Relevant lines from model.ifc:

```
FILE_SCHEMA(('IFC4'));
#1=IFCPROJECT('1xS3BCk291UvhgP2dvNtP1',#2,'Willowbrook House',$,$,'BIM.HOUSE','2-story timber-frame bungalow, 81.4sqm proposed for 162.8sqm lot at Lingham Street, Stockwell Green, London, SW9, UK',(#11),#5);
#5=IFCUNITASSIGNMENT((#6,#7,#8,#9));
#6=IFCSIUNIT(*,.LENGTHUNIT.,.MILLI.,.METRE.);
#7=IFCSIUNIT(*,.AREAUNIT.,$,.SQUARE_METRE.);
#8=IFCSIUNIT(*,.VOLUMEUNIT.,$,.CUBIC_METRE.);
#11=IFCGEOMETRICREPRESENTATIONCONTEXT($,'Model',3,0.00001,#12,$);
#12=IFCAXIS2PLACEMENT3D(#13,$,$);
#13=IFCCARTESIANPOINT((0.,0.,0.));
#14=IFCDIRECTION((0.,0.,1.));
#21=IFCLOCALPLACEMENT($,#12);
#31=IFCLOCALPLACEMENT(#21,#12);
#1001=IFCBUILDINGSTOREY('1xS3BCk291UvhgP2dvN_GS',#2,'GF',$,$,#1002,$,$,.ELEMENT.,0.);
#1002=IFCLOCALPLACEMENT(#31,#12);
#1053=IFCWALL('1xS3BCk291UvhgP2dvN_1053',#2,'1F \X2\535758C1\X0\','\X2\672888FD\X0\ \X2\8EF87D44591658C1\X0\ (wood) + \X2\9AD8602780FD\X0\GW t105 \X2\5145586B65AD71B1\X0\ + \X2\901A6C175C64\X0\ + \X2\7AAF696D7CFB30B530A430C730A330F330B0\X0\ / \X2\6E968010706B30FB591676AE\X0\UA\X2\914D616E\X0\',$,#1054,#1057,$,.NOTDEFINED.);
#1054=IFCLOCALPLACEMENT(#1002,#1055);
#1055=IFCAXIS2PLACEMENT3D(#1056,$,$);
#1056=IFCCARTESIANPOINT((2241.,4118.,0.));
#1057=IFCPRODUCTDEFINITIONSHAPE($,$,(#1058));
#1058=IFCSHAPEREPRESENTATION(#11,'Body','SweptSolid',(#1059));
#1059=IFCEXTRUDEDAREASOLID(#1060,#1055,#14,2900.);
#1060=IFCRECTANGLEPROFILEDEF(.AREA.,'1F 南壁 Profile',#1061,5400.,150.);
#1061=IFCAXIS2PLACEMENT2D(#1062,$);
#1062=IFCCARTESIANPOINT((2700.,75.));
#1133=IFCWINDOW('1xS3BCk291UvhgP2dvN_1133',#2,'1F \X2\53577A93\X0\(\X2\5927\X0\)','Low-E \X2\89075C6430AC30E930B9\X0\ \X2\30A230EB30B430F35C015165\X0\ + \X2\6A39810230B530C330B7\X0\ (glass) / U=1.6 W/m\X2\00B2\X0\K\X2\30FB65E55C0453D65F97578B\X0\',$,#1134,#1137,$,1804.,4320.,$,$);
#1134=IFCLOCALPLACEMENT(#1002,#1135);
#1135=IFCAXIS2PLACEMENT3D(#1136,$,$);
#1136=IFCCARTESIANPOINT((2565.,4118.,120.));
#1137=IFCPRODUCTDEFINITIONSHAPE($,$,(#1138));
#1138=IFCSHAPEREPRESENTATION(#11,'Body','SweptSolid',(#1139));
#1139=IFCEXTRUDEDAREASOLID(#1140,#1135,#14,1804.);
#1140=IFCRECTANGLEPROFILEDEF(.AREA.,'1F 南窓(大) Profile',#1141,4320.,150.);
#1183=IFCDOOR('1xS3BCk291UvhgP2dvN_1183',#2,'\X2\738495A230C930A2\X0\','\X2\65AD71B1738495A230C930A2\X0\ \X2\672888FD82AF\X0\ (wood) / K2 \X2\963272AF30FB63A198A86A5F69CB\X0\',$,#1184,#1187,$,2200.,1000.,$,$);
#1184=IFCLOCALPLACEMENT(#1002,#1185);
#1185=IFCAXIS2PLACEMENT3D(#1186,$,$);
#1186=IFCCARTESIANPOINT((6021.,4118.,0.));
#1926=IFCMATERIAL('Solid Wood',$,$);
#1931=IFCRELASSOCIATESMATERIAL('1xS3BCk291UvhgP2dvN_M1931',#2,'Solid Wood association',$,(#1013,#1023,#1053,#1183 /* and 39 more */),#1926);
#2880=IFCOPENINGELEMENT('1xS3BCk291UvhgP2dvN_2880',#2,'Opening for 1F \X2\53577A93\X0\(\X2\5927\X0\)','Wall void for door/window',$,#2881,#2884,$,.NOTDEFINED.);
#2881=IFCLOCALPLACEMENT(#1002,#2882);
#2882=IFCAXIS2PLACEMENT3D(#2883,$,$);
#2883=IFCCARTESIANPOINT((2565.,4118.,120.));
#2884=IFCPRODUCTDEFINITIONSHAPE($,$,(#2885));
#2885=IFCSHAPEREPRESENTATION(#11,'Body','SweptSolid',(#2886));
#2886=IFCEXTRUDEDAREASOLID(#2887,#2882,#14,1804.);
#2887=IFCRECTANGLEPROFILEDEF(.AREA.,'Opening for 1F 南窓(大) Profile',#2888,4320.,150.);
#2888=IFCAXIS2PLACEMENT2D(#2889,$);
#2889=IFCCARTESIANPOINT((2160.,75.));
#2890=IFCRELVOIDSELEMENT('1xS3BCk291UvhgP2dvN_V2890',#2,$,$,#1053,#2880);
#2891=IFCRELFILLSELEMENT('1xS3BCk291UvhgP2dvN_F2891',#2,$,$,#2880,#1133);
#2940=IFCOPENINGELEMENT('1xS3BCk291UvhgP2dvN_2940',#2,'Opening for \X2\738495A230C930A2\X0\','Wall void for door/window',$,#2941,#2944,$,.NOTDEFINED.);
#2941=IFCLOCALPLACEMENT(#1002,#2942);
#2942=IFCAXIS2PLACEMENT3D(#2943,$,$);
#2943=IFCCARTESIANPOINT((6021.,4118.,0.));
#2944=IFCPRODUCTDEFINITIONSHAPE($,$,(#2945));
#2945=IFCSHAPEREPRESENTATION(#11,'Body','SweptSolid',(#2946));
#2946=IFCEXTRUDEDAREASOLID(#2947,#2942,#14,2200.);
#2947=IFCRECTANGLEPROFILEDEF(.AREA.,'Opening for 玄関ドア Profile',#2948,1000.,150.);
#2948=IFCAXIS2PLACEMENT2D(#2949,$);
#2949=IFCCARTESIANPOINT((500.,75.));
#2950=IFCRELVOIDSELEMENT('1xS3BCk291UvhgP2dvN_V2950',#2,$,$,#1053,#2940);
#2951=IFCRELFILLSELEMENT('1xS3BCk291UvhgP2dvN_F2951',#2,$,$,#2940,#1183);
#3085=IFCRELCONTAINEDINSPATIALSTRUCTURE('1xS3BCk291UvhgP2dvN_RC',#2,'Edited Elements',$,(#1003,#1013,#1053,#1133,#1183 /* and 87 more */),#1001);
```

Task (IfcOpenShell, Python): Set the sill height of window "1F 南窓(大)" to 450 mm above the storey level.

```python
import numpy as np
import ifcopenshell
import ifcopenshell.api.geometry
import ifcopenshell.geom
import ifcopenshell.util.element
import ifcopenshell.util.placement
import ifcopenshell.util.shape
import ifcopenshell.util.unit

model = ifcopenshell.open("model.ifc")
unit_scale = ifcopenshell.util.unit.calculate_unit_scale(model)

window = model.by_guid("1xS3BCk291UvhgP2dvN_1133")
opening = window.FillsVoids[0].RelatingOpeningElement
storey = ifcopenshell.util.element.get_container(window, ifc_class="IfcBuildingStorey")
level = ifcopenshell.util.placement.get_local_placement(storey.ObjectPlacement)[2, 3]

# The opening's origin need not be at the sill, so measure its lowest point.
shape = ifcopenshell.geom.create_shape(ifcopenshell.geom.settings(), opening)
bottom = ifcopenshell.util.shape.get_shape_bottom_elevation(shape, shape.geometry) / unit_scale
dz = level + 0.45 / unit_scale - bottom

shift = np.array([0.0, 0.0, dz])
# The window is not placed relative to its opening, so move both.
for product in (opening, window):
    matrix = ifcopenshell.util.placement.get_local_placement(product.ObjectPlacement)
    matrix[:3, 3] += shift
    ifcopenshell.api.geometry.edit_object_placement(model, product=product, matrix=matrix, is_si=False)

print(f"moved by {dz * unit_scale:+.3f} m")

model.write("model_rev.ifc")
```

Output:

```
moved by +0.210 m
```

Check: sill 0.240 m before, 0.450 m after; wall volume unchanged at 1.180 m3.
